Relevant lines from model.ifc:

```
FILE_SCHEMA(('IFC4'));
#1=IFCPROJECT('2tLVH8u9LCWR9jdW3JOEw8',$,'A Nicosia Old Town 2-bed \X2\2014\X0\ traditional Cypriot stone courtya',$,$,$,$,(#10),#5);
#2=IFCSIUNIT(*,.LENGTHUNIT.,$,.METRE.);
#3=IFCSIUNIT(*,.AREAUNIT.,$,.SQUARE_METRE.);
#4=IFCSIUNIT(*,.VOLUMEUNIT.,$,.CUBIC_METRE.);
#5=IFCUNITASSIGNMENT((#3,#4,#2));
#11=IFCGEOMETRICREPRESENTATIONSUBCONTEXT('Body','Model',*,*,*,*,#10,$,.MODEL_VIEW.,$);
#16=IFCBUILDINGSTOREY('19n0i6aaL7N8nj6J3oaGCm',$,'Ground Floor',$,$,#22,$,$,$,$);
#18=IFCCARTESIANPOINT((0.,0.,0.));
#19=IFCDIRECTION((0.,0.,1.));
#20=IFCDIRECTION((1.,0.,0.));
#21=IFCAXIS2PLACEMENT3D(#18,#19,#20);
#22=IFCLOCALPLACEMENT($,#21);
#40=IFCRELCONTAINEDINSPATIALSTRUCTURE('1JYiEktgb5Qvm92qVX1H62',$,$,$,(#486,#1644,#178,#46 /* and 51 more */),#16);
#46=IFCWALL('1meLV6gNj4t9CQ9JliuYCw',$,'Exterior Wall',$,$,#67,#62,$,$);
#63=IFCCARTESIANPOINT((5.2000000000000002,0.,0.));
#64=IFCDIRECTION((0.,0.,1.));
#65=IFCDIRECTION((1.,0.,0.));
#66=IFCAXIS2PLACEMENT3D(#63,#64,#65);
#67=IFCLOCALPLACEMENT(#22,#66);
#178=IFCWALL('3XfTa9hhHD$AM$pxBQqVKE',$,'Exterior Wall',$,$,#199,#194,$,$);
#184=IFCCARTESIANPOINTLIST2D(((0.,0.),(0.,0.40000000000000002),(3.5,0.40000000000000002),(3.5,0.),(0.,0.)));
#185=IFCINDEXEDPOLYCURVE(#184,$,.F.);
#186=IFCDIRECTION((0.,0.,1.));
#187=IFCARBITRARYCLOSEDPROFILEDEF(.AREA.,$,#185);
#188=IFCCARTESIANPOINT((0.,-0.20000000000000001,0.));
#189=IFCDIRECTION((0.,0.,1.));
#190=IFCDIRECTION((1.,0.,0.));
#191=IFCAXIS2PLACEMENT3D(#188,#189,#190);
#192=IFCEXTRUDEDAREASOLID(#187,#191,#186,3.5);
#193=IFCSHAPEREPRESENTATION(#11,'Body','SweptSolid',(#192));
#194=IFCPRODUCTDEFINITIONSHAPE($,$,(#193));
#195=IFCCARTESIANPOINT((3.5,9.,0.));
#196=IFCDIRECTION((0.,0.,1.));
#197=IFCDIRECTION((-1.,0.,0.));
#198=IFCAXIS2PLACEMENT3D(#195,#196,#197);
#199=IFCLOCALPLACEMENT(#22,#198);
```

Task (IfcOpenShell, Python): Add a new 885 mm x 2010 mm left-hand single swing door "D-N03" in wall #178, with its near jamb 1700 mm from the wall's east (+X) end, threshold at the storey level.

```python
import numpy as np
import ifcopenshell
import ifcopenshell.api.feature
import ifcopenshell.api.geometry
import ifcopenshell.api.root
import ifcopenshell.api.spatial
import ifcopenshell.geom
import ifcopenshell.util.element
import ifcopenshell.util.placement
import ifcopenshell.util.representation
import ifcopenshell.util.shape
import ifcopenshell.util.unit

model = ifcopenshell.open("model.ifc")
unit_scale = ifcopenshell.util.unit.calculate_unit_scale(model)
settings = ifcopenshell.geom.settings()


def volume(element):
    """Net volume in cubic metres, openings subtracted."""
    shape = ifcopenshell.geom.create_shape(settings, element)
    return ifcopenshell.util.shape.get_volume(shape.geometry)


wall = model.by_guid("3XfTa9hhHD$AM$pxBQqVKE")
storey = ifcopenshell.util.element.get_container(wall, ifc_class="IfcBuildingStorey")
context = ifcopenshell.util.representation.get_context(model, "Model", "Body", "MODEL_VIEW")
before = volume(wall)

width, height, from_end, sill = 0.885, 2.01, 1.7, 0.0  # metres

# The wall runs along its own X axis, and the end named is its -X end.
wall_shape = ifcopenshell.geom.create_shape(settings, wall)
x, y, z = ifcopenshell.util.shape.get_vertices(wall_shape.geometry).T
start = x.min() + from_end
face, thickness = float(y.min()), float(y.max() - y.min())
wall_matrix = ifcopenshell.util.placement.get_local_placement(wall.ObjectPlacement)
level = ifcopenshell.util.placement.get_local_placement(storey.ObjectPlacement)[2, 3]


def in_wall(x, y):
    """Placement at x, y metres in the wall's axes, at sill height."""
    matrix = wall_matrix.copy()
    matrix[:, 3] = wall_matrix @ np.array([x / unit_scale, y / unit_scale, 0.0, 1.0])
    matrix[2, 3] = level + sill / unit_scale
    return matrix


# Opening: a box that overshoots both wall faces by 50 mm.
opening = ifcopenshell.api.root.create_entity(model, ifc_class="IfcOpeningElement", predefined_type="OPENING")
box = ifcopenshell.api.geometry.add_wall_representation(
    model, context=context, length=width, height=height, thickness=thickness + 0.1
)
ifcopenshell.api.geometry.assign_representation(model, product=opening, representation=box)
ifcopenshell.api.geometry.edit_object_placement(model, product=opening, matrix=in_wall(start, face - 0.05), is_si=False)
ifcopenshell.api.feature.add_feature(model, feature=opening, element=wall)

door = ifcopenshell.api.root.create_entity(model, ifc_class="IfcDoor", name="D-N03", predefined_type="DOOR")
door.OverallWidth, door.OverallHeight = width / unit_scale, height / unit_scale
door.OperationType = "SINGLE_SWING_LEFT"
body = ifcopenshell.api.geometry.add_door_representation(
    model,
    context=context,
    overall_width=door.OverallWidth,
    overall_height=door.OverallHeight,
    operation_type="SINGLE_SWING_LEFT",
    lining_properties={"LiningDepth": thickness / unit_scale, "ThresholdDepth": thickness / unit_scale},
)
ifcopenshell.api.geometry.assign_representation(model, product=door, representation=body)
ifcopenshell.api.spatial.assign_container(model, products=[door], relating_structure=storey)
ifcopenshell.api.feature.add_filling(model, opening=opening, element=door)

# The lining spans the wall, so the door starts at the wall face.
ifcopenshell.api.geometry.edit_object_placement(model, product=door, matrix=in_wall(start, face), is_si=False)

after = volume(wall)

print(f"wall volume {before:.3f} -> {after:.3f} m3")

model.write("model-out.ifc")
```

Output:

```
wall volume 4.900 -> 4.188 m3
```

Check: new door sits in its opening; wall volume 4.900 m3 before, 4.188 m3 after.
